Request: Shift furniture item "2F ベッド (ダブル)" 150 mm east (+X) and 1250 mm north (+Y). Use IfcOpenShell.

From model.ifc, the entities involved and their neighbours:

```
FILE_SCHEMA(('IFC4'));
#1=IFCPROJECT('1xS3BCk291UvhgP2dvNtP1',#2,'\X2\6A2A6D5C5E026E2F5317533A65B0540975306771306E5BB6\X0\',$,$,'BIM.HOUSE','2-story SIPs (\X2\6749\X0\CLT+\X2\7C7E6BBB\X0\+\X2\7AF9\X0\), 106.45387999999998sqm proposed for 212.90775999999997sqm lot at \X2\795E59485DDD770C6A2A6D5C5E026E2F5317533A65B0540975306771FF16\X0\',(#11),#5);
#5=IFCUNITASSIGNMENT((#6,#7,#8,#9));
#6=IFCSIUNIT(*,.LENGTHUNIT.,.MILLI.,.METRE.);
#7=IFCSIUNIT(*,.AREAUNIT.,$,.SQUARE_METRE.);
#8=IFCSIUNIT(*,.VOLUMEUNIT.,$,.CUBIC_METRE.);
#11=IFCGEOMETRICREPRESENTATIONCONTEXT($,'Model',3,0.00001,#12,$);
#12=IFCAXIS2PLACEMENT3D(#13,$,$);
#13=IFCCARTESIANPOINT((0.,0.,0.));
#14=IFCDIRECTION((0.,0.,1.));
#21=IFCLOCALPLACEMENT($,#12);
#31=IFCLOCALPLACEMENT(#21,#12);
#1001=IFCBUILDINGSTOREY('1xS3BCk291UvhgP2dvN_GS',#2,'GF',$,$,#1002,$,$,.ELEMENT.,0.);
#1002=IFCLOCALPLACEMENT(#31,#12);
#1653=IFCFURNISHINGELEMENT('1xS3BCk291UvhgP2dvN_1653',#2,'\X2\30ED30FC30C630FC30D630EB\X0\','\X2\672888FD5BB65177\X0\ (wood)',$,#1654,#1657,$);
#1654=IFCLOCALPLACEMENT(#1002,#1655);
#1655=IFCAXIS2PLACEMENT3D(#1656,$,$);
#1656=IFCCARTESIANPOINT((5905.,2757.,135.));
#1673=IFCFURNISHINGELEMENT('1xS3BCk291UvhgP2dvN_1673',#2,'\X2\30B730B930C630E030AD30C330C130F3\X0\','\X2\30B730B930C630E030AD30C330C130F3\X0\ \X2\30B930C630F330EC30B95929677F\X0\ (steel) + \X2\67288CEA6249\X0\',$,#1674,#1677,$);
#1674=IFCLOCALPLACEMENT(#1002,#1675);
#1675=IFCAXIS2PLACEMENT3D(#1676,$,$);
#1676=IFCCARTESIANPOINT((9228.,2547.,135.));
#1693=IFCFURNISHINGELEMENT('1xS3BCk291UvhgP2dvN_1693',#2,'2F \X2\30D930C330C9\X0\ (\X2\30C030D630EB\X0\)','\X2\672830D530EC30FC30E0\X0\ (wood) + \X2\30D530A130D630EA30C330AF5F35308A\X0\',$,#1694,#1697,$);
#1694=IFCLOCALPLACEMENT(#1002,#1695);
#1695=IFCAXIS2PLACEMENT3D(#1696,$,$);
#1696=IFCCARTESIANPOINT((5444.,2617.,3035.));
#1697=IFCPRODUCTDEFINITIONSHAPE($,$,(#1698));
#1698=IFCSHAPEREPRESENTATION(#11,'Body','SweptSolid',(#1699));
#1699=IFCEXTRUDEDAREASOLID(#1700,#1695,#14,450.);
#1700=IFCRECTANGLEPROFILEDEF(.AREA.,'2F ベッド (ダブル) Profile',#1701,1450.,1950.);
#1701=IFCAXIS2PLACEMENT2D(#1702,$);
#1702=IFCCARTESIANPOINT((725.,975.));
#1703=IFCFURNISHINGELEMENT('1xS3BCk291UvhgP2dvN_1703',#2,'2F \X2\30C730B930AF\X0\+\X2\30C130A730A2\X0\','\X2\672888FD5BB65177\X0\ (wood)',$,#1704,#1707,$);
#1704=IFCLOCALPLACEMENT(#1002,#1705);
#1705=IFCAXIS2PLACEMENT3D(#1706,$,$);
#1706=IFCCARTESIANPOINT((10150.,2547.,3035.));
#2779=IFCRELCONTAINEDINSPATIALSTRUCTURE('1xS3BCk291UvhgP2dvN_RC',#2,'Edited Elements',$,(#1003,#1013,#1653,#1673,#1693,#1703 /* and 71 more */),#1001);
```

```python
import ifcopenshell
import ifcopenshell.api.geometry
import ifcopenshell.util.placement
import ifcopenshell.util.unit

model = ifcopenshell.open("model.ifc")
unit_scale = ifcopenshell.util.unit.calculate_unit_scale(model)

item = model.by_guid("1xS3BCk291UvhgP2dvN_1693")
matrix = ifcopenshell.util.placement.get_local_placement(item.ObjectPlacement)
matrix[0, 3] += 0.15 / unit_scale
matrix[1, 3] += 1.25 / unit_scale
ifcopenshell.api.geometry.edit_object_placement(model, product=item, matrix=matrix, is_si=False)

print(ifcopenshell.util.placement.get_local_placement(item.ObjectPlacement).round(3) + 0.0)

model.write("model_v2.ifc")
```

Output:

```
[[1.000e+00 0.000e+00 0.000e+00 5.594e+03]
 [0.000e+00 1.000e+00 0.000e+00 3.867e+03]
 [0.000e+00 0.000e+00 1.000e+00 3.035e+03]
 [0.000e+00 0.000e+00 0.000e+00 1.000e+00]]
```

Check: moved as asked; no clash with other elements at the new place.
